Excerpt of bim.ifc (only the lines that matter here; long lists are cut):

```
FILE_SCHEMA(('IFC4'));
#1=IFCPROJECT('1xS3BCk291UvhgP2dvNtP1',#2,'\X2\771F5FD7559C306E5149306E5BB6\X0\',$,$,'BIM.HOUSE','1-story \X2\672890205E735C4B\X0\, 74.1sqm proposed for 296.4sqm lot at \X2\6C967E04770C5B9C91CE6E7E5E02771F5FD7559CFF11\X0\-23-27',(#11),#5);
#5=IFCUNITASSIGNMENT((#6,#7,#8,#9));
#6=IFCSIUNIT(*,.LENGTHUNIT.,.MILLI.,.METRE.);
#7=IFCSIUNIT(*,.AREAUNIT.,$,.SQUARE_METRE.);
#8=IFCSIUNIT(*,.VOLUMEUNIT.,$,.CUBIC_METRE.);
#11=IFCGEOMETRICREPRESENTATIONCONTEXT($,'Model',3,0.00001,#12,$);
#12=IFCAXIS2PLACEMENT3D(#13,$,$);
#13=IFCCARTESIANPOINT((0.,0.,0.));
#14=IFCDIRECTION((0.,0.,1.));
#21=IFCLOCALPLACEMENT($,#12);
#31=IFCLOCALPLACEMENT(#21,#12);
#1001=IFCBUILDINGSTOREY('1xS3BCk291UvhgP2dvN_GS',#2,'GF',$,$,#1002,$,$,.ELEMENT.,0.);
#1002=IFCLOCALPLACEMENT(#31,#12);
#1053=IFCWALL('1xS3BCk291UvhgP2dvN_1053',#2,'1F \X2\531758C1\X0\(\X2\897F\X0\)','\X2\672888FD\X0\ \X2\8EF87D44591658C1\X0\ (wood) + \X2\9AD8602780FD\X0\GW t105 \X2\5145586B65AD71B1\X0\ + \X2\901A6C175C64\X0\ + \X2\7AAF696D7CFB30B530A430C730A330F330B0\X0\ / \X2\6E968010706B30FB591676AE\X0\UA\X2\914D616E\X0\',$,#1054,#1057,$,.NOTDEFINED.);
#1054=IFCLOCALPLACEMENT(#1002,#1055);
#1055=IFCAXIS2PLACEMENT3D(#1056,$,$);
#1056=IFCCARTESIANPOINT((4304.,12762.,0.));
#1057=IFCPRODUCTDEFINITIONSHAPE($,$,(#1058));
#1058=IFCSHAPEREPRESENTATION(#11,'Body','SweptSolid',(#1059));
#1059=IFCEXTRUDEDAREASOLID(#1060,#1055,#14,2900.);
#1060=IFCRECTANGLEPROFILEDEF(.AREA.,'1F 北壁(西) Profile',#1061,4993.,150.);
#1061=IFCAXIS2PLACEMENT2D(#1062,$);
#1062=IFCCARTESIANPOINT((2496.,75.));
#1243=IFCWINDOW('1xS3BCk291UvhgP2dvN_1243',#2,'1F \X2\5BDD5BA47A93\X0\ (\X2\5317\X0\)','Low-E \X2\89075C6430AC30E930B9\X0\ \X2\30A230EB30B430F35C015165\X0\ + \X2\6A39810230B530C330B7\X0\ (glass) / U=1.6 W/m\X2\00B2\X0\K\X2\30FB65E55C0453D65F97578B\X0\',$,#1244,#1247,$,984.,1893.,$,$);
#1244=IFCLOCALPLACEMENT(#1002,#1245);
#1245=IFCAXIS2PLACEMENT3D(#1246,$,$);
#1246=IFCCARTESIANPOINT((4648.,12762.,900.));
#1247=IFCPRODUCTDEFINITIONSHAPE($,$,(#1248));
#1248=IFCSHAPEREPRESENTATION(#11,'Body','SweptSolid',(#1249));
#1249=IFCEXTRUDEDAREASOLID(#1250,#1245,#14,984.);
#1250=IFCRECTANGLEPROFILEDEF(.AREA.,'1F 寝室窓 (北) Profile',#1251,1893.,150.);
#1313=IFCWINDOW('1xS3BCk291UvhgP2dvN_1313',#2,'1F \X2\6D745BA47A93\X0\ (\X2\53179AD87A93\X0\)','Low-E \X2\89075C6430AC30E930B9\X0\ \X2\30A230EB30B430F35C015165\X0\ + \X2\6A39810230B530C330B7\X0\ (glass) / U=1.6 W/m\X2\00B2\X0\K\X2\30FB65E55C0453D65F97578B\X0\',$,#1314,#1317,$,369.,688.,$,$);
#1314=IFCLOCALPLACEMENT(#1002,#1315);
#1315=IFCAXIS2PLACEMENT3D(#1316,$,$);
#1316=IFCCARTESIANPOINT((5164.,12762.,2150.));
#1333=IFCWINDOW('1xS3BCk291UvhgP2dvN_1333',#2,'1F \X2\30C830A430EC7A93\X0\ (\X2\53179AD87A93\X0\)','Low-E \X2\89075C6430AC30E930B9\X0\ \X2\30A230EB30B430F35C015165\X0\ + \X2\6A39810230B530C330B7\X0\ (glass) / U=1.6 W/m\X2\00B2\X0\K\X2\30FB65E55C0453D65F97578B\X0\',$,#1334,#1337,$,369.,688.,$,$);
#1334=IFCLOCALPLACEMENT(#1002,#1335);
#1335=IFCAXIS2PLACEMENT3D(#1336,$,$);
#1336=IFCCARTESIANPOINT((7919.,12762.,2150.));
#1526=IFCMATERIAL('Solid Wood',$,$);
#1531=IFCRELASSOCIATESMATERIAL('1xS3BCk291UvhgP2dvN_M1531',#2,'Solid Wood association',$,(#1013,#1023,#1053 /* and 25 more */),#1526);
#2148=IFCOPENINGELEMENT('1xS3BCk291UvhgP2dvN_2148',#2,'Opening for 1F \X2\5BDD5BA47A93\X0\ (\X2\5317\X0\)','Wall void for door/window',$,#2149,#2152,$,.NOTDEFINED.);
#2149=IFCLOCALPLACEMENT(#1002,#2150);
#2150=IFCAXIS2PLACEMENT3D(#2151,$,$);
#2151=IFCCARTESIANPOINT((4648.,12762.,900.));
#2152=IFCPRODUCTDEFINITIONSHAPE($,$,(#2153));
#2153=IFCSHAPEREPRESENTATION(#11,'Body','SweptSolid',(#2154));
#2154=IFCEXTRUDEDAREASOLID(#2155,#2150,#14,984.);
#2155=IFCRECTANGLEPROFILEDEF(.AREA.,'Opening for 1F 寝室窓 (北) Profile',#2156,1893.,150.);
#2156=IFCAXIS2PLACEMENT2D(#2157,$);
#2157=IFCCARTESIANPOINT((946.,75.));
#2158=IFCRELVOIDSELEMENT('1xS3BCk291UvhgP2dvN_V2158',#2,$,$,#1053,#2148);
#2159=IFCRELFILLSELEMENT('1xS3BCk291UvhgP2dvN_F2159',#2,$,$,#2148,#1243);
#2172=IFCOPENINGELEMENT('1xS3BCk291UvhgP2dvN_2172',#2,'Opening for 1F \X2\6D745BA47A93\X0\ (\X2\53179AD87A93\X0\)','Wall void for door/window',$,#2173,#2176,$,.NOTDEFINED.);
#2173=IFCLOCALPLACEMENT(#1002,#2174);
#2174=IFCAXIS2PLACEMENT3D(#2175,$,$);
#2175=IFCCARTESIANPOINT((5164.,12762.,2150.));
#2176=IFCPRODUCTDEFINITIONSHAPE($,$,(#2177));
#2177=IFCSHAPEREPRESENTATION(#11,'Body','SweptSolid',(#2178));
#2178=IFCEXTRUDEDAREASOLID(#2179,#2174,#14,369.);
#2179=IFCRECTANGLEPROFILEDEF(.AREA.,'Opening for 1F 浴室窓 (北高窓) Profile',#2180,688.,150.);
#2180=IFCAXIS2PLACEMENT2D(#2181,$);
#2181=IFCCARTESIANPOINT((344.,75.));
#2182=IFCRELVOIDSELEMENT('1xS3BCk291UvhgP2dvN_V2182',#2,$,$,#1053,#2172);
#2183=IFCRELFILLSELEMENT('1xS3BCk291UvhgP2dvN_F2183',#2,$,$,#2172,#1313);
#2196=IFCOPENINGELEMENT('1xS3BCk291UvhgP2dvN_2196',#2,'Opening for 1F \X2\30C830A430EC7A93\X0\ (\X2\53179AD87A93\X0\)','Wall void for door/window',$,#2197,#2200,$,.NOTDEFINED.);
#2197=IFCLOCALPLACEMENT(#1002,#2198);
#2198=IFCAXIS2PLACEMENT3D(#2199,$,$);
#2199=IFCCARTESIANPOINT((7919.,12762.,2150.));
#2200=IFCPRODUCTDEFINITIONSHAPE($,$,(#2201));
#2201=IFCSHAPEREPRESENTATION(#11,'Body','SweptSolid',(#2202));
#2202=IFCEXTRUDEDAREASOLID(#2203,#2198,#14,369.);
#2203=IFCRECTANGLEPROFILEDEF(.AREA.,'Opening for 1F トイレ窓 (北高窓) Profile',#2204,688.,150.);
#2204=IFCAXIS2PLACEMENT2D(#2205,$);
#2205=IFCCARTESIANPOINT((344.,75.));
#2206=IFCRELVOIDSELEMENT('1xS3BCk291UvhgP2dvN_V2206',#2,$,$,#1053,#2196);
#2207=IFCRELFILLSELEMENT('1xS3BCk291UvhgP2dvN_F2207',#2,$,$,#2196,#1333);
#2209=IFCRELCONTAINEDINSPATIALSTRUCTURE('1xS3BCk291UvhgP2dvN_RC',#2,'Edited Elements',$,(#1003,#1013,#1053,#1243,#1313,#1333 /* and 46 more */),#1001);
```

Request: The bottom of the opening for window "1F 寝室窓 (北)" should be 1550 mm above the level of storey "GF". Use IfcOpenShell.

```python
import numpy as np
import ifcopenshell
import ifcopenshell.api.geometry
import ifcopenshell.geom
import ifcopenshell.util.element
import ifcopenshell.util.placement
import ifcopenshell.util.shape
import ifcopenshell.util.unit

model = ifcopenshell.open("bim.ifc")
unit_scale = ifcopenshell.util.unit.calculate_unit_scale(model)

window = model.by_guid("1xS3BCk291UvhgP2dvN_1243")
opening = window.FillsVoids[0].RelatingOpeningElement
storey = ifcopenshell.util.element.get_container(window, ifc_class="IfcBuildingStorey")
level = ifcopenshell.util.placement.get_local_placement(storey.ObjectPlacement)[2, 3]

# The opening's origin need not be at the sill, so measure its lowest point.
shape = ifcopenshell.geom.create_shape(ifcopenshell.geom.settings(), opening)
bottom = ifcopenshell.util.shape.get_shape_bottom_elevation(shape, shape.geometry) / unit_scale
dz = level + 1550.0 - bottom

shift = np.array([0.0, 0.0, dz])
# The window is not placed relative to its opening, so move both.
for product in (opening, window):
    matrix = ifcopenshell.util.placement.get_local_placement(product.ObjectPlacement)
    matrix[:3, 3] += shift
    ifcopenshell.api.geometry.edit_object_placement(model, product=product, matrix=matrix, is_si=False)

print(f"moved by {dz * unit_scale:+.3f} m")

model.write("bim_rev.ifc")
```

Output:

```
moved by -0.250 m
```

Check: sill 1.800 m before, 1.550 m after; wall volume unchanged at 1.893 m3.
